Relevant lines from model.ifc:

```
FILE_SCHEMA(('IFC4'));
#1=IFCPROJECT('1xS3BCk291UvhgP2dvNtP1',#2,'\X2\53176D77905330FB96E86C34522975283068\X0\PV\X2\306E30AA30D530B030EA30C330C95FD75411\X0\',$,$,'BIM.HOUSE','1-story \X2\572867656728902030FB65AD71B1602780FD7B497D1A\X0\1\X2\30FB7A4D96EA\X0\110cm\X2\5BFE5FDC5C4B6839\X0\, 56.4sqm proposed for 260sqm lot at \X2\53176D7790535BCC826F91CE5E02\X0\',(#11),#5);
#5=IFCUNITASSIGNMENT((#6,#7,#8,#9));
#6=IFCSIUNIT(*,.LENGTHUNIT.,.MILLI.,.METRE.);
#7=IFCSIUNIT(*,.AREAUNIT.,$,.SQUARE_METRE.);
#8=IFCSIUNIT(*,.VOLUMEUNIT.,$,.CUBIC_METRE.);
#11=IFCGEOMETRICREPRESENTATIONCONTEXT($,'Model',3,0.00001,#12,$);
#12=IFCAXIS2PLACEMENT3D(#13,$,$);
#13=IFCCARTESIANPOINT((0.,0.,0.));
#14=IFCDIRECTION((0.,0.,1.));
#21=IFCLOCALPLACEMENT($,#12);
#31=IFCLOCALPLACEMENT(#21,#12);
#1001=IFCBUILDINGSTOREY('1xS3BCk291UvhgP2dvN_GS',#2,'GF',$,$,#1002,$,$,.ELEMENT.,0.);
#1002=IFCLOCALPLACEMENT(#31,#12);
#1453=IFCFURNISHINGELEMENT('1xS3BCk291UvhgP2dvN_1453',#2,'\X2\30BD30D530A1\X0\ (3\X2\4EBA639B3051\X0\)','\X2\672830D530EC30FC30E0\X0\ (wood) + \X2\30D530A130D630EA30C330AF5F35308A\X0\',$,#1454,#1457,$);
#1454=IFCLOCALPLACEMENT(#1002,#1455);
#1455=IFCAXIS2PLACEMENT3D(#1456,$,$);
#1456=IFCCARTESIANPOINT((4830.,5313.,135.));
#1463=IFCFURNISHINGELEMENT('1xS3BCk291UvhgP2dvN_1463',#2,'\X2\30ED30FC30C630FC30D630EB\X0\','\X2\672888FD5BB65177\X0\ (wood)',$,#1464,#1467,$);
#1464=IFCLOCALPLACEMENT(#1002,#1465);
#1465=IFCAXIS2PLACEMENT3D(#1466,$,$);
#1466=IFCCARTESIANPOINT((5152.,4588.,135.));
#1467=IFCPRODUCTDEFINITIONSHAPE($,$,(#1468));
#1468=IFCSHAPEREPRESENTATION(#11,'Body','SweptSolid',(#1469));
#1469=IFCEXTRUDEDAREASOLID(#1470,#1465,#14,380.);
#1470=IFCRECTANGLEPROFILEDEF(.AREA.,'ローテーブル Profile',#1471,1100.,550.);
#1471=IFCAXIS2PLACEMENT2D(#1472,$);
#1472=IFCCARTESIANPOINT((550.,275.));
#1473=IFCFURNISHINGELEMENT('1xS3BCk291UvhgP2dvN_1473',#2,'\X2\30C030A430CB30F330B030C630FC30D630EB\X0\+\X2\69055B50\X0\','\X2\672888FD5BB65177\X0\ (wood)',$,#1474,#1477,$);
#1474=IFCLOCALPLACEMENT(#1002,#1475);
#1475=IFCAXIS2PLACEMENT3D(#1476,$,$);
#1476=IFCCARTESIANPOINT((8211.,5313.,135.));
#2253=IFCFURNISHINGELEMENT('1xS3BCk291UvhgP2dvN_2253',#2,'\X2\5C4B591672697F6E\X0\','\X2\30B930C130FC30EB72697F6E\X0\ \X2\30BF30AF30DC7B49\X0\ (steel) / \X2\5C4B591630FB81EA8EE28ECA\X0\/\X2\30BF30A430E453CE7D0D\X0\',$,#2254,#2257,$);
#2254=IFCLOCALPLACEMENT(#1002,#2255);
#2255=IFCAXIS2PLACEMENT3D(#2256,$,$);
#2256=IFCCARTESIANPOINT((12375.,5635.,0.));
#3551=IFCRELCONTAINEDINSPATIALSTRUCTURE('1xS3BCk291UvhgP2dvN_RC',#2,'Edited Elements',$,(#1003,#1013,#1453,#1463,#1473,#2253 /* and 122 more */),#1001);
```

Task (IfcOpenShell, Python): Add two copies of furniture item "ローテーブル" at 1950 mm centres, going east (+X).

```python
import numpy as np
import ifcopenshell
import ifcopenshell.api.geometry
import ifcopenshell.api.root
import ifcopenshell.util.element
import ifcopenshell.util.placement

model = ifcopenshell.open("model.ifc")


def reuse_history(source, copy):
    """copy_class also copies each property set's owner history, people and application; keep the originals."""
    for rel in copy.IsDefinedBy:
        if rel.is_a("IfcRelDefinesByProperties") and (history := rel.RelatingPropertyDefinition.OwnerHistory):
            rel.RelatingPropertyDefinition.OwnerHistory = source.OwnerHistory
            ifcopenshell.util.element.remove_deep2(model, history)


source = model.by_guid("1xS3BCk291UvhgP2dvN_1463")
base = ifcopenshell.util.placement.get_local_placement(source.ObjectPlacement)
step = np.array([1.0, 0.0, 0.0]) * 1950.0

for i in range(1, 3):
    copy = ifcopenshell.api.root.copy_class(model, product=source)
    copy.Representation = ifcopenshell.util.element.copy_deep(
        model, source.Representation, exclude=["IfcGeometricRepresentationContext", "IfcRepresentationMap"]
    )
    reuse_history(source, copy)
    matrix = base.copy()
    matrix[:3, 3] += i * step
    print("added at", matrix[:3, 3].round(3) + 0.0)
    ifcopenshell.api.geometry.edit_object_placement(model, product=copy, matrix=matrix, is_si=False)

model.write("model_updated.ifc")
```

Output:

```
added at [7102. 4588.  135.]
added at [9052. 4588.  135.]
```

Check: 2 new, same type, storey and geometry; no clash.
